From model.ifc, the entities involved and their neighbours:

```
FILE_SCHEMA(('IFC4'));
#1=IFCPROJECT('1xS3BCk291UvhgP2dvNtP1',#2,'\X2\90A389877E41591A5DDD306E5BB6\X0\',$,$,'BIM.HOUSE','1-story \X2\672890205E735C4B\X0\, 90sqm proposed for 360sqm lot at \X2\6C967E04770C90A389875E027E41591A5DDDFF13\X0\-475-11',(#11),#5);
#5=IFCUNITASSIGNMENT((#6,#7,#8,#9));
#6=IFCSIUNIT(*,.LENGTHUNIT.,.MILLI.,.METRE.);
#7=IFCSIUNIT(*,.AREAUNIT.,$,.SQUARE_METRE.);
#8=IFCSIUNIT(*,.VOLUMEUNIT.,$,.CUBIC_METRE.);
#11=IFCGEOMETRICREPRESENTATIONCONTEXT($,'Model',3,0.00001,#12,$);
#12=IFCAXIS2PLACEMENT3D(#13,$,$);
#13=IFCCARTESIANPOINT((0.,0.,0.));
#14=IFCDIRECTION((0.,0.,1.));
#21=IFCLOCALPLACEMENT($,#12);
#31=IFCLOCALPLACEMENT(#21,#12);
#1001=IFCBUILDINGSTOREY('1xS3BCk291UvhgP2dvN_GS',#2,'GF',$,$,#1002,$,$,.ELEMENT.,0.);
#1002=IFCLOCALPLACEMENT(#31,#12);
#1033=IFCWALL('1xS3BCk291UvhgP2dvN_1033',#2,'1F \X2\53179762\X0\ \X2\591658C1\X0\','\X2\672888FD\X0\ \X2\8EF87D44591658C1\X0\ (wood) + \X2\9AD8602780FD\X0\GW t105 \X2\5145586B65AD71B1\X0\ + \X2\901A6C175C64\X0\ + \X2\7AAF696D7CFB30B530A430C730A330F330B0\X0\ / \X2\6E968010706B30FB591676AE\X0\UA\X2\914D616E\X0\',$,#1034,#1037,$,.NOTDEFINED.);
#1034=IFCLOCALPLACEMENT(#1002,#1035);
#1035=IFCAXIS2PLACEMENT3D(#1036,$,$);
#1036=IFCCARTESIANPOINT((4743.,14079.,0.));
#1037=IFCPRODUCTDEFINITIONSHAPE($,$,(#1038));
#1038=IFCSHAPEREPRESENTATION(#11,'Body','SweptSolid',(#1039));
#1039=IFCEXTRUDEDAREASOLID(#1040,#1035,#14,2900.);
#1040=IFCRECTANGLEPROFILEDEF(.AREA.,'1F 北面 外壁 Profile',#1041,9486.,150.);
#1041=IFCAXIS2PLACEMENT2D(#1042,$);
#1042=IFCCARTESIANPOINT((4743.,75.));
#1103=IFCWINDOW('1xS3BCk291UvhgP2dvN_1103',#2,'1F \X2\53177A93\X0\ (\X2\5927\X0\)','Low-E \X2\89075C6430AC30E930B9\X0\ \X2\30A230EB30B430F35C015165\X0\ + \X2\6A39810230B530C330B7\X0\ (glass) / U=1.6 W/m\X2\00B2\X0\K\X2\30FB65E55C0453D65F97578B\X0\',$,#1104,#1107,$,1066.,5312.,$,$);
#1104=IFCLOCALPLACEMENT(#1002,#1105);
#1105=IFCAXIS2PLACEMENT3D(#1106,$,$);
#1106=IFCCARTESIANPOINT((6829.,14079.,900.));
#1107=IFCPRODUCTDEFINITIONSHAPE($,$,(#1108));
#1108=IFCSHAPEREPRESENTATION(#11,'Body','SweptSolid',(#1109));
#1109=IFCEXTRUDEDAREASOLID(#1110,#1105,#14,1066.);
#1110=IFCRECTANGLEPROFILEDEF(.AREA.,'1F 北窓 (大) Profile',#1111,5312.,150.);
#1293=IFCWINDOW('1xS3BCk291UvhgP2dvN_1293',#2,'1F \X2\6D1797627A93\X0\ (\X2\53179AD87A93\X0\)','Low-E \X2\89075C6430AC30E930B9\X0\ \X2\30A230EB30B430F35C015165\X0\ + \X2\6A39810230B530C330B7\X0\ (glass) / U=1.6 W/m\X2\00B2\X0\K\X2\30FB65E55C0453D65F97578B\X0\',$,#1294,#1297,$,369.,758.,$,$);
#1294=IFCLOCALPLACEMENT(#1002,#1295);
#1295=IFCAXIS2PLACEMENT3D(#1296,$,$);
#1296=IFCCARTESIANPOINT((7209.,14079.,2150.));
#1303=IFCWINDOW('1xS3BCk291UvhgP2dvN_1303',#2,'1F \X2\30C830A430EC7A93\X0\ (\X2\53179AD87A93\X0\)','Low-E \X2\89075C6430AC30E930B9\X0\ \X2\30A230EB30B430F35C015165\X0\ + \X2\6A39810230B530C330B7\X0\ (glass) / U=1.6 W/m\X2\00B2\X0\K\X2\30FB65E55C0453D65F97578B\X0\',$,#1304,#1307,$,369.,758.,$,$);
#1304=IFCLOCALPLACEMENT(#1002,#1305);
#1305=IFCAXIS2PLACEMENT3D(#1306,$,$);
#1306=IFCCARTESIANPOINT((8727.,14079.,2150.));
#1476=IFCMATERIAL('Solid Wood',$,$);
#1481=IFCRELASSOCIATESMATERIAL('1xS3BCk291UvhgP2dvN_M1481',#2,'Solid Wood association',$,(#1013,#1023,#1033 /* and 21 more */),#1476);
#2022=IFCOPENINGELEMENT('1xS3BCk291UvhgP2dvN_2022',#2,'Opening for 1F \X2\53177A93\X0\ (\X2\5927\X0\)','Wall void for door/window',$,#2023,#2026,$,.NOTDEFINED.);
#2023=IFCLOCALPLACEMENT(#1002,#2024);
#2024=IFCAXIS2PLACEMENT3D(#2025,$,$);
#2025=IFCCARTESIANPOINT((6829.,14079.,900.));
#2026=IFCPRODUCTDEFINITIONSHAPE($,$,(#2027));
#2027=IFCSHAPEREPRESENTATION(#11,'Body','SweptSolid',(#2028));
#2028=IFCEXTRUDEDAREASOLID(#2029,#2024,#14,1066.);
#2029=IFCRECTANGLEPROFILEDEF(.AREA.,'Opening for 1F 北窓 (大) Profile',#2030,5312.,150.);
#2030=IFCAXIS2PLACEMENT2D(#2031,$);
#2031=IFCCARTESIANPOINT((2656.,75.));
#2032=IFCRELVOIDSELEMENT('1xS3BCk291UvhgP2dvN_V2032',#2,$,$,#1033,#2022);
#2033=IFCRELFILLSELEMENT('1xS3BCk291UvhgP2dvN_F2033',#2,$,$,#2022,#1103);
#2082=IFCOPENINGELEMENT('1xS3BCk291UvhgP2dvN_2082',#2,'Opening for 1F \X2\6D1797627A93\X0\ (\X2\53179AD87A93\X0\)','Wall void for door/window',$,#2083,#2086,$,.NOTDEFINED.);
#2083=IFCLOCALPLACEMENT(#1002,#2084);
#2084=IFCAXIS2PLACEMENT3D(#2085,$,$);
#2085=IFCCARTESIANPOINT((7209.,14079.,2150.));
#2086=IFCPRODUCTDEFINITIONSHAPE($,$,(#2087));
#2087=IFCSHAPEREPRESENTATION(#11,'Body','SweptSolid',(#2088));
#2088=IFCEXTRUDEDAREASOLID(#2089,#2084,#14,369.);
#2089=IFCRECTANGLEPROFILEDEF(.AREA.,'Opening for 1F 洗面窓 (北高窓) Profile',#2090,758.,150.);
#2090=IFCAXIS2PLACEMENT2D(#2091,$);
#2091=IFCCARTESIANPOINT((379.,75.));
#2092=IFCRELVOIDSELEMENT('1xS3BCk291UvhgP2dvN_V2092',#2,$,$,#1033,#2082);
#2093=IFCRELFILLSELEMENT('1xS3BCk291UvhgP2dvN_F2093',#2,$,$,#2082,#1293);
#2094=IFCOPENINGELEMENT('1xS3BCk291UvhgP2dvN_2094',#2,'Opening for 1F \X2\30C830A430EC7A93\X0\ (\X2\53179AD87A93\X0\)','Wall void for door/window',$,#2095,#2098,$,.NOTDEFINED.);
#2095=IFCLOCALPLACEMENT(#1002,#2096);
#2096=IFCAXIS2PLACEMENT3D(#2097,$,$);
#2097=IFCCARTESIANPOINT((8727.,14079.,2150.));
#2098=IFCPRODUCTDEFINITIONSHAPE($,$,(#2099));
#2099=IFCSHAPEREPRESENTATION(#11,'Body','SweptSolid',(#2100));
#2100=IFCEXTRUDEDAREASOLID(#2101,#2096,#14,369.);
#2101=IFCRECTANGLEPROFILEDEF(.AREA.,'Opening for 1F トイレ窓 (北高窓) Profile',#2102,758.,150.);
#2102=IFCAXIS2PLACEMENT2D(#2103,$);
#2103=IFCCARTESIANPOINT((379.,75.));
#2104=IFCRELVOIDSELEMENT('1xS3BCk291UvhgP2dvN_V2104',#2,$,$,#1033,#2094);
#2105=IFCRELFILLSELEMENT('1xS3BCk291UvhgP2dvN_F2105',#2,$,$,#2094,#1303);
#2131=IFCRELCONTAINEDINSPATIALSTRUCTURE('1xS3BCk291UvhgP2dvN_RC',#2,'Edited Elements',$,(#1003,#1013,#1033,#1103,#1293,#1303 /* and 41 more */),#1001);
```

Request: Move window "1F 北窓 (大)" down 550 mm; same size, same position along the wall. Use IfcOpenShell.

```python
import numpy as np
import ifcopenshell
import ifcopenshell.api.geometry
import ifcopenshell.util.placement
import ifcopenshell.util.unit

model = ifcopenshell.open("model.ifc")
unit_scale = ifcopenshell.util.unit.calculate_unit_scale(model)

window = model.by_guid("1xS3BCk291UvhgP2dvN_1103")
opening = window.FillsVoids[0].RelatingOpeningElement
dz = -550.0

shift = np.array([0.0, 0.0, dz])
# The window is not placed relative to its opening, so move both.
for product in (opening, window):
    matrix = ifcopenshell.util.placement.get_local_placement(product.ObjectPlacement)
    matrix[:3, 3] += shift
    ifcopenshell.api.geometry.edit_object_placement(model, product=product, matrix=matrix, is_si=False)

print(f"moved by {dz * unit_scale:+.3f} m")

model.write("model_v2.ifc")
```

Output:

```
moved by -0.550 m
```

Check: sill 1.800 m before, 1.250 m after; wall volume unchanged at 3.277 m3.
